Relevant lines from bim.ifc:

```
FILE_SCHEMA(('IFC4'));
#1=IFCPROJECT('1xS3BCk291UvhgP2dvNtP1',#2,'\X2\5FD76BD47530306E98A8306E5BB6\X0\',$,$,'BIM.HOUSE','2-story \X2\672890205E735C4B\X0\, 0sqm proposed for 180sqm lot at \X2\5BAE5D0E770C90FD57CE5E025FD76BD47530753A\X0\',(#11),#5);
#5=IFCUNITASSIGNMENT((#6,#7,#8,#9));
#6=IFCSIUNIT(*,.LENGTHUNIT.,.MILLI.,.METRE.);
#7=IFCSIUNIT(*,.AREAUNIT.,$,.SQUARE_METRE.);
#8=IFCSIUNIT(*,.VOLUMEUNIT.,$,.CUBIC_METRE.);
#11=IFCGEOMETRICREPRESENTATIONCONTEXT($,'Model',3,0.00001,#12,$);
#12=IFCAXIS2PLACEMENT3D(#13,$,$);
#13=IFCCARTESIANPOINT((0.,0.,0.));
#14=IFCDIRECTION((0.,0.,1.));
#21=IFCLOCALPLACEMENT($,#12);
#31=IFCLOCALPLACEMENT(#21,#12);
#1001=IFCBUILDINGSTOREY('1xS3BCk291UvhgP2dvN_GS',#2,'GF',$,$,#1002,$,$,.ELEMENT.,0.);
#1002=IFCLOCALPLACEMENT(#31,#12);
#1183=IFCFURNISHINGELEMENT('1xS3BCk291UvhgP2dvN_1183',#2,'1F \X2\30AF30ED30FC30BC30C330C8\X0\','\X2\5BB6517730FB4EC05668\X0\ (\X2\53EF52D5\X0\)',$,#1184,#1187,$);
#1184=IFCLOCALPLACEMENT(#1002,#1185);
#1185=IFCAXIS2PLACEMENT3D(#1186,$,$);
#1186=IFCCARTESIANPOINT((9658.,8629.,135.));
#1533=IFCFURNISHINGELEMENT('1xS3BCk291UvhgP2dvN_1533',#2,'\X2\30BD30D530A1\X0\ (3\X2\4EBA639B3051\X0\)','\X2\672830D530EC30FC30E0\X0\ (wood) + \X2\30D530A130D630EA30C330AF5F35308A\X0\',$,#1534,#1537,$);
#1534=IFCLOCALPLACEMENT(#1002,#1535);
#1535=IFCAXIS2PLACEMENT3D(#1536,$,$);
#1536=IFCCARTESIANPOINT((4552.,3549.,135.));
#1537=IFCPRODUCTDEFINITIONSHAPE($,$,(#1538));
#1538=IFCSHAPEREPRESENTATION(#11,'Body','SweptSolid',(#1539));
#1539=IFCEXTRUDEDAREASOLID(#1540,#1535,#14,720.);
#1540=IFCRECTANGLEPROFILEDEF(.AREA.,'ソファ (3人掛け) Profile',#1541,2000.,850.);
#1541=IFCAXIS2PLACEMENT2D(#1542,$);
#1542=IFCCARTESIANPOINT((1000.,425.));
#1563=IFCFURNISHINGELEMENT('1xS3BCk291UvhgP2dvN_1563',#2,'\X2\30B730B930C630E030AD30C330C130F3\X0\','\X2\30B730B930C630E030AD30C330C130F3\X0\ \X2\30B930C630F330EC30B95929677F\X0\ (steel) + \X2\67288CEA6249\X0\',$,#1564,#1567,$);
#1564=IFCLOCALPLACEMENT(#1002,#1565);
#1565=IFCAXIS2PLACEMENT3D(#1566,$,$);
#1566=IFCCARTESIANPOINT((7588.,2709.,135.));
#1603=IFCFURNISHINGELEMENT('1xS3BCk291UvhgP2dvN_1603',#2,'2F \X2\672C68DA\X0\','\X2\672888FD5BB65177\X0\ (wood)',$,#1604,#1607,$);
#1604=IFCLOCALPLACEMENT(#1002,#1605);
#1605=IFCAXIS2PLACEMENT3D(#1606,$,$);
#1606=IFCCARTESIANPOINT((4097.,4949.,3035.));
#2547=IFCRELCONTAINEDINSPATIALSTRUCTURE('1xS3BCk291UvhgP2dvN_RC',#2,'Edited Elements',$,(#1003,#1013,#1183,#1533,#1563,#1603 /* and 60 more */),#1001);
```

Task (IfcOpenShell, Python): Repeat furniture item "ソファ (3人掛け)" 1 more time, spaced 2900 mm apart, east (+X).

```python
import numpy as np
import ifcopenshell
import ifcopenshell.api.geometry
import ifcopenshell.api.root
import ifcopenshell.util.element
import ifcopenshell.util.placement
import ifcopenshell.util.unit

model = ifcopenshell.open("bim.ifc")
unit_scale = ifcopenshell.util.unit.calculate_unit_scale(model)


def reuse_history(source, copy):
    """copy_class also copies each property set's owner history, people and application; keep the originals."""
    for rel in copy.IsDefinedBy:
        if rel.is_a("IfcRelDefinesByProperties") and (history := rel.RelatingPropertyDefinition.OwnerHistory):
            rel.RelatingPropertyDefinition.OwnerHistory = source.OwnerHistory
            ifcopenshell.util.element.remove_deep2(model, history)


source = model.by_id(1533)
base = ifcopenshell.util.placement.get_local_placement(source.ObjectPlacement)
step = np.array([1.0, 0.0, 0.0]) * 2.9 / unit_scale

for i in range(1, 2):
    copy = ifcopenshell.api.root.copy_class(model, product=source)
    copy.Representation = ifcopenshell.util.element.copy_deep(
        model, source.Representation, exclude=["IfcGeometricRepresentationContext", "IfcRepresentationMap"]
    )
    reuse_history(source, copy)
    matrix = base.copy()
    matrix[:3, 3] += i * step
    print("added at", matrix[:3, 3].round(3) + 0.0)
    ifcopenshell.api.geometry.edit_object_placement(model, product=copy, matrix=matrix, is_si=False)

model.write("bim_rev.ifc")
```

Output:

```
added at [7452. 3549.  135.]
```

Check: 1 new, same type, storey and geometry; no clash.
